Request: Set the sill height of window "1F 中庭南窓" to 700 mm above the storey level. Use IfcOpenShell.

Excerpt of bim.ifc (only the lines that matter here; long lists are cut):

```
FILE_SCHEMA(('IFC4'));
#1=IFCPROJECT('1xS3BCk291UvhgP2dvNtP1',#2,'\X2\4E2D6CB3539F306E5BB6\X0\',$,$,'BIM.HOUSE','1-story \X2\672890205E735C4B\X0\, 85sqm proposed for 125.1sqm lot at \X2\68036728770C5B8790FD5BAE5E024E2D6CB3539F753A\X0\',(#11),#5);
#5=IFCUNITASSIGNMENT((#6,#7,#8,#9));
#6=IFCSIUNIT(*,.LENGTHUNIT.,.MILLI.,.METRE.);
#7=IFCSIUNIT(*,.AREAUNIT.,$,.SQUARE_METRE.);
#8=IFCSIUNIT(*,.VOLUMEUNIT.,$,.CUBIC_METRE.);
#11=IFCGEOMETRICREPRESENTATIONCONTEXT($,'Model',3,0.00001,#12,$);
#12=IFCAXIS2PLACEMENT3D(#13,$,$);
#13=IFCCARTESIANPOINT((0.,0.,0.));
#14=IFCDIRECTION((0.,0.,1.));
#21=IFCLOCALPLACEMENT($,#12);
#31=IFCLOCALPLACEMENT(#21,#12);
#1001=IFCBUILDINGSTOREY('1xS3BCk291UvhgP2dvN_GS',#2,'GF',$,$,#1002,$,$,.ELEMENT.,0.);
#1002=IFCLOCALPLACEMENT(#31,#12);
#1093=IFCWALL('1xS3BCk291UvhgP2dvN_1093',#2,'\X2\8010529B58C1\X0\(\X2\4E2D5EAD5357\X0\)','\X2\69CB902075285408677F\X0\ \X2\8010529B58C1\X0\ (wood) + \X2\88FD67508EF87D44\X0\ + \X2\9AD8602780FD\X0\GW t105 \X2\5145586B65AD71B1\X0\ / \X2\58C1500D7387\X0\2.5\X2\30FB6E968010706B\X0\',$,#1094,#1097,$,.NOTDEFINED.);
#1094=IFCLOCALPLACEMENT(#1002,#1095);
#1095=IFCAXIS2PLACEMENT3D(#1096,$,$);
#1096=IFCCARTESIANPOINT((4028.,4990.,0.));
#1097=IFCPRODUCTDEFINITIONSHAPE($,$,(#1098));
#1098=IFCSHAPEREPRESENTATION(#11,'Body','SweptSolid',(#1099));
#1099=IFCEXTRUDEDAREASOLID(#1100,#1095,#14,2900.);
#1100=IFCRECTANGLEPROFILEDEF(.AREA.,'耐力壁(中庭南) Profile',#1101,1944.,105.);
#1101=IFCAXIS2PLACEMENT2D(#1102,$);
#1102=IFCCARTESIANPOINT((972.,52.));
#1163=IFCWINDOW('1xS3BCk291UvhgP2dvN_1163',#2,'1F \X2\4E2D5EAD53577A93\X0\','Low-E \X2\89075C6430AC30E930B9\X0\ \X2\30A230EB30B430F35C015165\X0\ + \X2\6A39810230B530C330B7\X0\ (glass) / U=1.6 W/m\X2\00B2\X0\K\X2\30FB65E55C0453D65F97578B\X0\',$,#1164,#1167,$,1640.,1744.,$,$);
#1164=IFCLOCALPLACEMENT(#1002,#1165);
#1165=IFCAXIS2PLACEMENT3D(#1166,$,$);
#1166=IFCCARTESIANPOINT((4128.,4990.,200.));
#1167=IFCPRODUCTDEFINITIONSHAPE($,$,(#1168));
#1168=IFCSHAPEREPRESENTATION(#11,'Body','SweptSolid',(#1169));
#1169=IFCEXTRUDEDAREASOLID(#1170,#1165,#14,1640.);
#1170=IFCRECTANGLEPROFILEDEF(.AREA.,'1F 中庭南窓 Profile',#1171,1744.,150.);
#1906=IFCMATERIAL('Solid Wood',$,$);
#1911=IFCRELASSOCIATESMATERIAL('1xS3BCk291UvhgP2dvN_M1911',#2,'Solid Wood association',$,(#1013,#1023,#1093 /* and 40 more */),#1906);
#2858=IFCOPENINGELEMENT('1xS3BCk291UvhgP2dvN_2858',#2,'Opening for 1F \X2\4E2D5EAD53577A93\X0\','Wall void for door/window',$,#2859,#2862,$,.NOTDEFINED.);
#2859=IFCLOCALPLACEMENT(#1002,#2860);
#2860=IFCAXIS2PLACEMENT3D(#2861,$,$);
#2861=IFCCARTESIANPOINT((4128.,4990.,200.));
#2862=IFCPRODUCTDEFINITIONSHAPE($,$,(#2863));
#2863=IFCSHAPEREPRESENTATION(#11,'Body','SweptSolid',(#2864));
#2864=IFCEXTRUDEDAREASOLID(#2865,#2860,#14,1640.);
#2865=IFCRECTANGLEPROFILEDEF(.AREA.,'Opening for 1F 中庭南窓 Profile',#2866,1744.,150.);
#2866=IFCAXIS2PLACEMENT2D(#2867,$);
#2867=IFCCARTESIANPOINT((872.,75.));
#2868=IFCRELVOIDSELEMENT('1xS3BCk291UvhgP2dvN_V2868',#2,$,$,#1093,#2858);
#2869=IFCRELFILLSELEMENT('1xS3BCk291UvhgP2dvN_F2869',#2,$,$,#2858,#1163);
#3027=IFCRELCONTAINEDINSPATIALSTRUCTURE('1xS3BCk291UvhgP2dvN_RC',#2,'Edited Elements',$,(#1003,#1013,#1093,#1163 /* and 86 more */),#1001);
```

```python
import numpy as np
import ifcopenshell
import ifcopenshell.api.geometry
import ifcopenshell.geom
import ifcopenshell.util.element
import ifcopenshell.util.placement
import ifcopenshell.util.shape
import ifcopenshell.util.unit

model = ifcopenshell.open("bim.ifc")
unit_scale = ifcopenshell.util.unit.calculate_unit_scale(model)

window = model.by_id(1163)
opening = window.FillsVoids[0].RelatingOpeningElement
storey = ifcopenshell.util.element.get_container(window, ifc_class="IfcBuildingStorey")
level = ifcopenshell.util.placement.get_local_placement(storey.ObjectPlacement)[2, 3]

# The opening's origin need not be at the sill, so measure its lowest point.
shape = ifcopenshell.geom.create_shape(ifcopenshell.geom.settings(), opening)
bottom = ifcopenshell.util.shape.get_shape_bottom_elevation(shape, shape.geometry) / unit_scale
dz = level + 700.0 - bottom

shift = np.array([0.0, 0.0, dz])
# The window is not placed relative to its opening, so move both.
for product in (opening, window):
    matrix = ifcopenshell.util.placement.get_local_placement(product.ObjectPlacement)
    matrix[:3, 3] += shift
    ifcopenshell.api.geometry.edit_object_placement(model, product=product, matrix=matrix, is_si=False)

print(f"moved by {dz * unit_scale:+.3f} m")

model.write("bim-out.ifc")
```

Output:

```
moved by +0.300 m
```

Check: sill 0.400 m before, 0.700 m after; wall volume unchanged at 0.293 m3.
